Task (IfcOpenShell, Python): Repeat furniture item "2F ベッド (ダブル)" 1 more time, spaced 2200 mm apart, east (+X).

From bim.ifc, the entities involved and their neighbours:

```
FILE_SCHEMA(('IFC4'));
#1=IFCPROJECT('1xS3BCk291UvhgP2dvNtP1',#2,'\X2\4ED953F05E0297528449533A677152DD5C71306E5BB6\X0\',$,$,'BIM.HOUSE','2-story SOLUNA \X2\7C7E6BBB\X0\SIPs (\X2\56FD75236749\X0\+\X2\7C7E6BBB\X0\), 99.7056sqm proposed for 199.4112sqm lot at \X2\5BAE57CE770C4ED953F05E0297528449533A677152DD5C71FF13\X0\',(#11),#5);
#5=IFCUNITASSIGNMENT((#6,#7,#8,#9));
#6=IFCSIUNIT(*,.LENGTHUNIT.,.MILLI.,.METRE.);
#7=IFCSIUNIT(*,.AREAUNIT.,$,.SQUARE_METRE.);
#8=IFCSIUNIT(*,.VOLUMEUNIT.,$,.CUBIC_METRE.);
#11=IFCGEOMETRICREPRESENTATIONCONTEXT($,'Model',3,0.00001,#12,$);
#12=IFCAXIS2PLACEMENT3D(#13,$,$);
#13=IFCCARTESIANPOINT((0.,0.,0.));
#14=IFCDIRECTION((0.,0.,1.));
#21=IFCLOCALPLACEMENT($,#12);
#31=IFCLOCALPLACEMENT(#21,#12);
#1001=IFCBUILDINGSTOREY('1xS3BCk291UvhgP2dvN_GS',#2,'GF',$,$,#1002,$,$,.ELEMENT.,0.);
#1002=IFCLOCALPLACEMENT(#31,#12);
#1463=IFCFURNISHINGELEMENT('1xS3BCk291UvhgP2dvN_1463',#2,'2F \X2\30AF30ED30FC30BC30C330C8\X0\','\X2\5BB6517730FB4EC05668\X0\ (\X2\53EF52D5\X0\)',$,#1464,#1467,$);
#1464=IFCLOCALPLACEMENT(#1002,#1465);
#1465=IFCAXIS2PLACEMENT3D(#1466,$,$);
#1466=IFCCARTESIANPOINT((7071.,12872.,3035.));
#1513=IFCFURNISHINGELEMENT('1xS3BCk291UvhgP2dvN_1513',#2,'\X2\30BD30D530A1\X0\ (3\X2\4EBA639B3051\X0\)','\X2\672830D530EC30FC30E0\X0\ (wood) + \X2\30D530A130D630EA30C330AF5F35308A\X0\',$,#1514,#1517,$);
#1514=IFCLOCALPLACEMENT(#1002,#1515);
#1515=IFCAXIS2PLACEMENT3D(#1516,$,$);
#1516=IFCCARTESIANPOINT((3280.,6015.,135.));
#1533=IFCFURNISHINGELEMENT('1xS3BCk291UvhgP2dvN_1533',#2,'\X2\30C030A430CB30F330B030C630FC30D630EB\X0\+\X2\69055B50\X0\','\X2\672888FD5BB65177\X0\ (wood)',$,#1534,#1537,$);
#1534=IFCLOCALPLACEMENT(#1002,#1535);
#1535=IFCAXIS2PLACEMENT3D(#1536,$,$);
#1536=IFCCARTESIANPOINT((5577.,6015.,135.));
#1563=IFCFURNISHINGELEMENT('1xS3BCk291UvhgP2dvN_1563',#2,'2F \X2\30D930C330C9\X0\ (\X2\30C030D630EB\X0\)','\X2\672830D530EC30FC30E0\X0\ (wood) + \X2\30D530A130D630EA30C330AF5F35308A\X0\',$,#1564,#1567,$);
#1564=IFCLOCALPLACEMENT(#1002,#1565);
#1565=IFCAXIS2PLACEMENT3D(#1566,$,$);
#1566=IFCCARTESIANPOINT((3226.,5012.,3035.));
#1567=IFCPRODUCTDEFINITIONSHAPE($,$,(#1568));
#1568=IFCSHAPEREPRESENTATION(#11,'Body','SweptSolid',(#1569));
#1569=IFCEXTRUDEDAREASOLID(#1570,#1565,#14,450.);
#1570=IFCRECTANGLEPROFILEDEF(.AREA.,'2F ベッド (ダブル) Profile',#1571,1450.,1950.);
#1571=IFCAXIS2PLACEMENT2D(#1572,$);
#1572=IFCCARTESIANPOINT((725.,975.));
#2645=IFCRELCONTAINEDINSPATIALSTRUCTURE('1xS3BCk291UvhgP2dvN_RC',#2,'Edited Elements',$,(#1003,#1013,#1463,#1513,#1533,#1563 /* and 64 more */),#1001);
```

```python
import numpy as np
import ifcopenshell
import ifcopenshell.api.geometry
import ifcopenshell.api.root
import ifcopenshell.util.element
import ifcopenshell.util.placement

model = ifcopenshell.open("bim.ifc")


def reuse_history(source, copy):
    """copy_class also copies each property set's owner history, people and application; keep the originals."""
    for rel in copy.IsDefinedBy:
        if rel.is_a("IfcRelDefinesByProperties") and (history := rel.RelatingPropertyDefinition.OwnerHistory):
            rel.RelatingPropertyDefinition.OwnerHistory = source.OwnerHistory
            ifcopenshell.util.element.remove_deep2(model, history)


source = model.by_id(1563)
base = ifcopenshell.util.placement.get_local_placement(source.ObjectPlacement)
step = np.array([1.0, 0.0, 0.0]) * 2200.0

for i in range(1, 2):
    copy = ifcopenshell.api.root.copy_class(model, product=source)
    copy.Representation = ifcopenshell.util.element.copy_deep(
        model, source.Representation, exclude=["IfcGeometricRepresentationContext", "IfcRepresentationMap"]
    )
    reuse_history(source, copy)
    matrix = base.copy()
    matrix[:3, 3] += i * step
    print("added at", matrix[:3, 3].round(3) + 0.0)
    ifcopenshell.api.geometry.edit_object_placement(model, product=copy, matrix=matrix, is_si=False)

model.write("bim_v2.ifc")
```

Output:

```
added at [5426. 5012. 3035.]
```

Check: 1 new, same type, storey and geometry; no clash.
